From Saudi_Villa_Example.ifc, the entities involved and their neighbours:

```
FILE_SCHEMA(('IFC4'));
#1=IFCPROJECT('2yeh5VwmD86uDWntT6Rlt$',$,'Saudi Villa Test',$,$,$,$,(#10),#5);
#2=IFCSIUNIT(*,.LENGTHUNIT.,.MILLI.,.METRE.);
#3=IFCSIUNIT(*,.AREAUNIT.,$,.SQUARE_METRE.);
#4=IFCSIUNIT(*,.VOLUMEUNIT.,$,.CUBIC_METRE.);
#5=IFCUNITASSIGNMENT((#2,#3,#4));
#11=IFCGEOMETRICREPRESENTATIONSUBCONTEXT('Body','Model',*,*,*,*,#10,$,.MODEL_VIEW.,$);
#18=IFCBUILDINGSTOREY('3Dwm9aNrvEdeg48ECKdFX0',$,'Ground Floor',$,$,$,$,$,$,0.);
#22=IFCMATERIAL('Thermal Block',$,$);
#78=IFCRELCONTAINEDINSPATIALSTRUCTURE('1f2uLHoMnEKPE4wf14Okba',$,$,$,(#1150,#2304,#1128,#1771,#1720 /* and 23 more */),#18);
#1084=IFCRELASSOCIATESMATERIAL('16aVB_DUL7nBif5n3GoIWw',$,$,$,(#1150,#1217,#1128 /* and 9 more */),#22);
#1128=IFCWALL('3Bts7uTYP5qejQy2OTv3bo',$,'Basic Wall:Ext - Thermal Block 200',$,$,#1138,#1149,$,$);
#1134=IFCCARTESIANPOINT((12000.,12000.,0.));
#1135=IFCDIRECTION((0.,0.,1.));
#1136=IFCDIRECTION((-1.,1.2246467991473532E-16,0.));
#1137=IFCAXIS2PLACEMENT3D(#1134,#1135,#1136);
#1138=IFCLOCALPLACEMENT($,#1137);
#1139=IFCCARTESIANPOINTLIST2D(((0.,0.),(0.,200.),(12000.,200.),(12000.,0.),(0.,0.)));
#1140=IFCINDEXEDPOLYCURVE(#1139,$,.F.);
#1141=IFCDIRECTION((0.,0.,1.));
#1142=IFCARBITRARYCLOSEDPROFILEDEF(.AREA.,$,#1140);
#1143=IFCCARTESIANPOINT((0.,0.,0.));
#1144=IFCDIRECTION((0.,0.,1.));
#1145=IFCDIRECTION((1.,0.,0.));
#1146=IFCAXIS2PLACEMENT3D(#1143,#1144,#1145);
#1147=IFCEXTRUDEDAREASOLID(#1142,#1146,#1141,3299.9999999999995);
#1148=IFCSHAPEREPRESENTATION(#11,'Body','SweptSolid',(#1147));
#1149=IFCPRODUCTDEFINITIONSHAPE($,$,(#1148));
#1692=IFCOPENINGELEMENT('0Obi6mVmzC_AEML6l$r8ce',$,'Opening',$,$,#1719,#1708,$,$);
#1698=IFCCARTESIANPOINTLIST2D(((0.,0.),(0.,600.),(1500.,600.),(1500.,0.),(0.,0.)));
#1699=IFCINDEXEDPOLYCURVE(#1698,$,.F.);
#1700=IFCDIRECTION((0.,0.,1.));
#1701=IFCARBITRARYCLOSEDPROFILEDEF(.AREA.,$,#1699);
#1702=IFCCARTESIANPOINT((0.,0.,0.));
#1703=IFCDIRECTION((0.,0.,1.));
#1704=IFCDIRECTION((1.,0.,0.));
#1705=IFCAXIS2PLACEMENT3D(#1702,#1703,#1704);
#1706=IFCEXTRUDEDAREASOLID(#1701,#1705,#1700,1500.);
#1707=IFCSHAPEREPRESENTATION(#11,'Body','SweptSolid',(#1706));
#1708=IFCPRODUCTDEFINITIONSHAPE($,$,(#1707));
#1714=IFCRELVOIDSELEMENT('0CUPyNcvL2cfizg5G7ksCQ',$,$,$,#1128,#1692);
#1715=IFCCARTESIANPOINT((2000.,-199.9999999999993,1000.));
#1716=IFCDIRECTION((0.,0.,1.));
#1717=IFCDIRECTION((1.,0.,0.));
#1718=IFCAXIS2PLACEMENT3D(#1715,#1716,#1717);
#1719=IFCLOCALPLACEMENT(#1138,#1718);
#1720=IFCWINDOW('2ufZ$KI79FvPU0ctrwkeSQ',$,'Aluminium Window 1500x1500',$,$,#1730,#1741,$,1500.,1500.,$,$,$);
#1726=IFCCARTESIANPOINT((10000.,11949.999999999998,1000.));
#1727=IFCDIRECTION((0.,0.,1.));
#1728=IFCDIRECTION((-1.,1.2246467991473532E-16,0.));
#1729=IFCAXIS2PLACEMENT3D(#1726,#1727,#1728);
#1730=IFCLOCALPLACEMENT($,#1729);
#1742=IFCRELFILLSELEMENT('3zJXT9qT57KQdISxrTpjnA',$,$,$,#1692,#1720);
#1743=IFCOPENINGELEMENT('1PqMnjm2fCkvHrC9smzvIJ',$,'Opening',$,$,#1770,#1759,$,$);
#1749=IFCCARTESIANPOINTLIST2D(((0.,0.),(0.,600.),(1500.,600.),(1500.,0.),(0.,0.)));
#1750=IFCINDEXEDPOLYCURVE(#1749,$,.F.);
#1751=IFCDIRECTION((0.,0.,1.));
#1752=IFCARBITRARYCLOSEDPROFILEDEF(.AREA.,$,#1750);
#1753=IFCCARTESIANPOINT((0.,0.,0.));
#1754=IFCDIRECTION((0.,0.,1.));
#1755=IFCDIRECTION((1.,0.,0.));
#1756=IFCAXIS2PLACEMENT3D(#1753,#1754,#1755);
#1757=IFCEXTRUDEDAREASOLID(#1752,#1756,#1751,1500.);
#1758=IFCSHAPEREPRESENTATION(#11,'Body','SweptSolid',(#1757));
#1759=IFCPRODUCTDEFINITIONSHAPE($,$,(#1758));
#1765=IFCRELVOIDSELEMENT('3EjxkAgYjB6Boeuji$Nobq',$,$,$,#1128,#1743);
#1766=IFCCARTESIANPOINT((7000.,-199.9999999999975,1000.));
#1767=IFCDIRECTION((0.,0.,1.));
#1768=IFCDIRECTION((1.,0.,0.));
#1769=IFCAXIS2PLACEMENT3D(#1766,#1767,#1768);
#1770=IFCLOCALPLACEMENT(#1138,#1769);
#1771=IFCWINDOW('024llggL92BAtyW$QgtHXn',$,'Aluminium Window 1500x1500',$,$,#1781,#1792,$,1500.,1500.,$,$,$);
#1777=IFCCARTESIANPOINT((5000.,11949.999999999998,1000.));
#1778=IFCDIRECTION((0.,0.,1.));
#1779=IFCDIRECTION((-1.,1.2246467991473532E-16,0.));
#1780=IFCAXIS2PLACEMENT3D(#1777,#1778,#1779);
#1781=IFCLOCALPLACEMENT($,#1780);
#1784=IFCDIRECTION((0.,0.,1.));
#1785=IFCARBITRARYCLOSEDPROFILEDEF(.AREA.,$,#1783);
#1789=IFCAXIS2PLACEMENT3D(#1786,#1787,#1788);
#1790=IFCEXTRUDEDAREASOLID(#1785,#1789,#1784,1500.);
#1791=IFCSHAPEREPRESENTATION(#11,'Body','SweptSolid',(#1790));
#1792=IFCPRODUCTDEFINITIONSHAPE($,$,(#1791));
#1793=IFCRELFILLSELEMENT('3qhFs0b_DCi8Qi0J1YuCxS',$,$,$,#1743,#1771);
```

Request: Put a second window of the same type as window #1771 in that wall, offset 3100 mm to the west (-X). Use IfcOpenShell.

```python
import ifcopenshell
import ifcopenshell.api.feature
import ifcopenshell.api.geometry
import ifcopenshell.api.root
import ifcopenshell.geom
import ifcopenshell.util.element
import ifcopenshell.util.placement
import ifcopenshell.util.shape
import ifcopenshell.util.unit

model = ifcopenshell.open("Saudi_Villa_Example.ifc")
unit_scale = ifcopenshell.util.unit.calculate_unit_scale(model)
settings = ifcopenshell.geom.settings()


def volume(element):
    """Net volume in cubic metres, openings subtracted."""
    shape = ifcopenshell.geom.create_shape(settings, element)
    return ifcopenshell.util.shape.get_volume(shape.geometry)


window = model.by_guid("024llggL92BAtyW$QgtHXn")
opening = window.FillsVoids[0].RelatingOpeningElement
wall = opening.VoidsElements[0].RelatingBuildingElement
before = volume(wall)
shift = ifcopenshell.util.placement.get_local_placement(wall.ObjectPlacement)[:3, 0] * 3.1 / unit_scale

# copy_class copies the void relationship, type, container and properties, but no geometry.
new_opening = ifcopenshell.api.root.copy_class(model, product=opening)
new_opening.Representation = ifcopenshell.util.element.copy_deep(
    model, opening.Representation, exclude=["IfcGeometricRepresentationContext", "IfcRepresentationMap"]
)
new_window = ifcopenshell.api.root.copy_class(model, product=window)
new_window.Representation = ifcopenshell.util.element.copy_deep(
    model, window.Representation, exclude=["IfcGeometricRepresentationContext", "IfcRepresentationMap"]
)
ifcopenshell.api.feature.add_filling(model, opening=new_opening, element=new_window)

for old, new in ((opening, new_opening), (window, new_window)):
    matrix = ifcopenshell.util.placement.get_local_placement(old.ObjectPlacement)
    matrix[:3, 3] += shift
    ifcopenshell.api.geometry.edit_object_placement(model, product=new, matrix=matrix, is_si=False)

after = volume(wall)

print(f"wall volume {before:.3f} -> {after:.3f} m3")

model.write("Saudi_Villa_Example_updated.ifc")
```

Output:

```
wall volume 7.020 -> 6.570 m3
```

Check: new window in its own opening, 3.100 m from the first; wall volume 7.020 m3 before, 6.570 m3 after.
